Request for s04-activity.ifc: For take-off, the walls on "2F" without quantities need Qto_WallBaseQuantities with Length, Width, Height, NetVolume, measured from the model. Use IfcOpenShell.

First a look at what the model holds.

```python
import ifcopenshell
import ifcopenshell.util.element
import ifcopenshell.util.unit

model = ifcopenshell.open("s04-activity.ifc")
print(model.schema)
for unit_type in ("LENGTHUNIT", "AREAUNIT", "VOLUMEUNIT"):
    print(unit_type, ifcopenshell.util.unit.calculate_unit_scale(model, unit_type))
storey = next(s for s in model.by_type("IfcBuildingStorey") if s.Name == "2F")
walls = [e for e in ifcopenshell.util.element.get_decomposition(storey) if e.is_a("IfcWall")]
for e in sorted(walls, key=lambda e: e.id()):
    print(e.id(), e.is_a(), e.Name, list(ifcopenshell.util.element.get_psets(e, qtos_only=True)), sep=" | ")
```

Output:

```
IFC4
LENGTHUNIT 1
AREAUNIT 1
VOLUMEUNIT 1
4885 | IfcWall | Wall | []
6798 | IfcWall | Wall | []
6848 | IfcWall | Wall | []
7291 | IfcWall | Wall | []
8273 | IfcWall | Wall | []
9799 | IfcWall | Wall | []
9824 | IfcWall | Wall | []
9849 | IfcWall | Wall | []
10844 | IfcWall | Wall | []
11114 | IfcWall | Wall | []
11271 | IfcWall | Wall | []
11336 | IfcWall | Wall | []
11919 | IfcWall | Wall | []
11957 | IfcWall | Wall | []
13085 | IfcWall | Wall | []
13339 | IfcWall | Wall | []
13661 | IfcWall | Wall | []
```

```python
import ifcopenshell
import ifcopenshell.api.pset
import ifcopenshell.geom
import ifcopenshell.util.element
import ifcopenshell.util.shape
import ifcopenshell.util.unit

model = ifcopenshell.open("s04-activity.ifc")
unit_scale = ifcopenshell.util.unit.calculate_unit_scale(model)
volume_scale = ifcopenshell.util.unit.calculate_unit_scale(model, "VOLUMEUNIT")
settings = ifcopenshell.geom.settings()

storey = next(s for s in model.by_type("IfcBuildingStorey") if s.Name == "2F")
walls = [e for e in ifcopenshell.util.element.get_decomposition(storey) if e.is_a("IfcWall")]

for e in sorted(walls, key=lambda e: e.id()):
    if ifcopenshell.util.element.get_psets(e, qtos_only=True, should_inherit=False):
        continue
    # Geometry comes back in metres, in the element's own axes.
    shape = ifcopenshell.geom.create_shape(settings, e)
    values = {
        "Length": ifcopenshell.util.shape.get_x(shape.geometry) / unit_scale,
        "Width": ifcopenshell.util.shape.get_y(shape.geometry) / unit_scale,
        "Height": ifcopenshell.util.shape.get_z(shape.geometry) / unit_scale,
        "NetVolume": ifcopenshell.util.shape.get_volume(shape.geometry) / volume_scale,
    }
    qto = ifcopenshell.api.pset.add_qto(model, product=e, name="Qto_WallBaseQuantities")
    ifcopenshell.api.pset.edit_qto(model, qto=qto, properties=values)
    print(e.id(), {k: round(v, 3) for k, v in values.items()})

model.write("s04-activity_updated.ifc")
```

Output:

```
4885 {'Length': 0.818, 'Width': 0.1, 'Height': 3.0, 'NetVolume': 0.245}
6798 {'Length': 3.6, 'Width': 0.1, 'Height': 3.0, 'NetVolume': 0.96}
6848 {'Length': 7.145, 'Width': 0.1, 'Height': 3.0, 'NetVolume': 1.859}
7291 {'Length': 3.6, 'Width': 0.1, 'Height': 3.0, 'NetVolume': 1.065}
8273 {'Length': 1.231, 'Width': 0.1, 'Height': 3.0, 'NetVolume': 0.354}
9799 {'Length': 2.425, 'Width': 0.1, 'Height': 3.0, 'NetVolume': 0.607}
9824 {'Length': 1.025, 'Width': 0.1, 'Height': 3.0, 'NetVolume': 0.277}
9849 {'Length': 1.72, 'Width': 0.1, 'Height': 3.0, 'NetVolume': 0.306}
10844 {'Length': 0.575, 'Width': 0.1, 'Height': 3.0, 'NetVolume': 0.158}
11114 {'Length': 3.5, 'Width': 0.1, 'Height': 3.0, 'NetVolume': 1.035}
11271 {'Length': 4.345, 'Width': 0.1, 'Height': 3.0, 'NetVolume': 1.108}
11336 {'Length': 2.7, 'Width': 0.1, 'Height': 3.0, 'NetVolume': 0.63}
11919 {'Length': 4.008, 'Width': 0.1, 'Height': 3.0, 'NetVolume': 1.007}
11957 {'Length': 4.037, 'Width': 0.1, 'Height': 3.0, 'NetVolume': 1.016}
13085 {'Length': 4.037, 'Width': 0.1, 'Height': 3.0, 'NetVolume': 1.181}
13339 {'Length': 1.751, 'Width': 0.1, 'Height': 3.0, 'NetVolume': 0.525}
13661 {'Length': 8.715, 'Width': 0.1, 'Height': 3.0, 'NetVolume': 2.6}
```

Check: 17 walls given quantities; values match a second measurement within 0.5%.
